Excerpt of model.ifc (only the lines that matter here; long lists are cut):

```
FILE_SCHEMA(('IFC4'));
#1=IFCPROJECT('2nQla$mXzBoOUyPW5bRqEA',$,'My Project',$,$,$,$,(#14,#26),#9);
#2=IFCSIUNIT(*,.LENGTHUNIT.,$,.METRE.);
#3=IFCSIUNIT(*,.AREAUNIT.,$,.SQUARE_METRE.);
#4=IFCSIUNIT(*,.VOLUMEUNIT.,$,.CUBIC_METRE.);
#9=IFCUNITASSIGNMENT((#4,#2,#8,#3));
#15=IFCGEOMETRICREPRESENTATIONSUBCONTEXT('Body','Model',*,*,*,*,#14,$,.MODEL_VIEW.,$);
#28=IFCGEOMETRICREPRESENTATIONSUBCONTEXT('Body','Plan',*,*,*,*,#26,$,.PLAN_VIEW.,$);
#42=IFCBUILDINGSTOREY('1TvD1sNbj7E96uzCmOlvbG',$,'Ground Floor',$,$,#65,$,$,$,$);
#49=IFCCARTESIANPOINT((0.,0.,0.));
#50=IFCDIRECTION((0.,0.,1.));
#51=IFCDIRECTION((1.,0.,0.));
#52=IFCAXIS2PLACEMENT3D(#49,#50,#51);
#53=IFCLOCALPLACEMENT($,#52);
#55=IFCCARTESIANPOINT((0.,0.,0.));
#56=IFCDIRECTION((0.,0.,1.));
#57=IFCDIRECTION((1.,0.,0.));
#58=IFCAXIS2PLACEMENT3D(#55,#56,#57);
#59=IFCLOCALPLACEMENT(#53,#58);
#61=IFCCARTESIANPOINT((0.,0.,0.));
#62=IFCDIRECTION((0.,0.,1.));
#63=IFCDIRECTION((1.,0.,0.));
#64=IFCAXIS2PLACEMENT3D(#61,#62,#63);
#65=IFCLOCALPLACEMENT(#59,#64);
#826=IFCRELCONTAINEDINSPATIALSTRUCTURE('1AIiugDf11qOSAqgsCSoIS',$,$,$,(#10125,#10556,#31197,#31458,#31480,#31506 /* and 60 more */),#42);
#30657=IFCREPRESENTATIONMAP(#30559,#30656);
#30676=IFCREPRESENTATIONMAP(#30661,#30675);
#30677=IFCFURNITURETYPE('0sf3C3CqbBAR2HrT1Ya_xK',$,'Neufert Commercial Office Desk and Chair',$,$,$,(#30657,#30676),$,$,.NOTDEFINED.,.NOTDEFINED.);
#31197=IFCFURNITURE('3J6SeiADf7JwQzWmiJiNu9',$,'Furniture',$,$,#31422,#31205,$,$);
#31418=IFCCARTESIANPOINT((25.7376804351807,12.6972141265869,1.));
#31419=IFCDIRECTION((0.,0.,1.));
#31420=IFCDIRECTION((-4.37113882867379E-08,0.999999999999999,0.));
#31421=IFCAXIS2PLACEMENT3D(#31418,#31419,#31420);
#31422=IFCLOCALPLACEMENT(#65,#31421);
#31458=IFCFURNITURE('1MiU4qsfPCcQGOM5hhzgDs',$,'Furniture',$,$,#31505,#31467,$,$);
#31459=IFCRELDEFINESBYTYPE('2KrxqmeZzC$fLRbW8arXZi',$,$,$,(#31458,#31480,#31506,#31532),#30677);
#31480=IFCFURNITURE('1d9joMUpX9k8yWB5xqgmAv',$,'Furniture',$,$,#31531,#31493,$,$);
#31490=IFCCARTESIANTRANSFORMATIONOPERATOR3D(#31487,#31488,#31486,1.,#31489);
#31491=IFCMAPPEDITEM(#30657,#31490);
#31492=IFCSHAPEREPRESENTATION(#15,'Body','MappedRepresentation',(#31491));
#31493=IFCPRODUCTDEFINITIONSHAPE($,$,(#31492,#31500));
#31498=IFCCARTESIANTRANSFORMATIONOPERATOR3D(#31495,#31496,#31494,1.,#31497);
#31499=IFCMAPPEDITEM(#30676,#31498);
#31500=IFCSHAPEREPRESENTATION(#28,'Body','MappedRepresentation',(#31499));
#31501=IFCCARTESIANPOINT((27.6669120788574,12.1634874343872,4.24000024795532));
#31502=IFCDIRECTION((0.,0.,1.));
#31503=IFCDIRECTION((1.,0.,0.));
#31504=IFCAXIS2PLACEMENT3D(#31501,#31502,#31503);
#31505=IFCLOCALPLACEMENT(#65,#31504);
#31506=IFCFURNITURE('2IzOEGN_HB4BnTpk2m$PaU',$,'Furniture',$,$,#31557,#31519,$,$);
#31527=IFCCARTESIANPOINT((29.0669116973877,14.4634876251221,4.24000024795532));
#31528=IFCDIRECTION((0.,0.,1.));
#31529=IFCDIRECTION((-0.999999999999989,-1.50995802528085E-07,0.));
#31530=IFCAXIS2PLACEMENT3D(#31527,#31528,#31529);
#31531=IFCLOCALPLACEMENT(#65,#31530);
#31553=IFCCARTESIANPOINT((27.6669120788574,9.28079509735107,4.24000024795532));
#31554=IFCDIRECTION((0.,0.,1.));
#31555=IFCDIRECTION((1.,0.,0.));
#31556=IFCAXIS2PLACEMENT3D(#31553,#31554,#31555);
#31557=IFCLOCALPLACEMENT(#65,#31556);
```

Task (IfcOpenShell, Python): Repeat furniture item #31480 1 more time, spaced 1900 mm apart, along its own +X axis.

```python
import ifcopenshell
import ifcopenshell.api.geometry
import ifcopenshell.api.root
import ifcopenshell.util.element
import ifcopenshell.util.placement

model = ifcopenshell.open("model.ifc")

source = model.by_guid("1d9joMUpX9k8yWB5xqgmAv")
base = ifcopenshell.util.placement.get_local_placement(source.ObjectPlacement)
step = base[:3, 0] * 1.9

for i in range(1, 2):
    copy = ifcopenshell.api.root.copy_class(model, product=source)
    copy.Representation = ifcopenshell.util.element.copy_deep(
        model, source.Representation, exclude=["IfcGeometricRepresentationContext", "IfcRepresentationMap"]
    )
    matrix = base.copy()
    matrix[:3, 3] += i * step
    print("added at", matrix[:3, 3].round(3) + 0.0)
    ifcopenshell.api.geometry.edit_object_placement(model, product=copy, matrix=matrix, is_si=False)

model.write("model_rev.ifc")
```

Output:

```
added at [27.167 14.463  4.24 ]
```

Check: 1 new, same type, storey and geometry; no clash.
